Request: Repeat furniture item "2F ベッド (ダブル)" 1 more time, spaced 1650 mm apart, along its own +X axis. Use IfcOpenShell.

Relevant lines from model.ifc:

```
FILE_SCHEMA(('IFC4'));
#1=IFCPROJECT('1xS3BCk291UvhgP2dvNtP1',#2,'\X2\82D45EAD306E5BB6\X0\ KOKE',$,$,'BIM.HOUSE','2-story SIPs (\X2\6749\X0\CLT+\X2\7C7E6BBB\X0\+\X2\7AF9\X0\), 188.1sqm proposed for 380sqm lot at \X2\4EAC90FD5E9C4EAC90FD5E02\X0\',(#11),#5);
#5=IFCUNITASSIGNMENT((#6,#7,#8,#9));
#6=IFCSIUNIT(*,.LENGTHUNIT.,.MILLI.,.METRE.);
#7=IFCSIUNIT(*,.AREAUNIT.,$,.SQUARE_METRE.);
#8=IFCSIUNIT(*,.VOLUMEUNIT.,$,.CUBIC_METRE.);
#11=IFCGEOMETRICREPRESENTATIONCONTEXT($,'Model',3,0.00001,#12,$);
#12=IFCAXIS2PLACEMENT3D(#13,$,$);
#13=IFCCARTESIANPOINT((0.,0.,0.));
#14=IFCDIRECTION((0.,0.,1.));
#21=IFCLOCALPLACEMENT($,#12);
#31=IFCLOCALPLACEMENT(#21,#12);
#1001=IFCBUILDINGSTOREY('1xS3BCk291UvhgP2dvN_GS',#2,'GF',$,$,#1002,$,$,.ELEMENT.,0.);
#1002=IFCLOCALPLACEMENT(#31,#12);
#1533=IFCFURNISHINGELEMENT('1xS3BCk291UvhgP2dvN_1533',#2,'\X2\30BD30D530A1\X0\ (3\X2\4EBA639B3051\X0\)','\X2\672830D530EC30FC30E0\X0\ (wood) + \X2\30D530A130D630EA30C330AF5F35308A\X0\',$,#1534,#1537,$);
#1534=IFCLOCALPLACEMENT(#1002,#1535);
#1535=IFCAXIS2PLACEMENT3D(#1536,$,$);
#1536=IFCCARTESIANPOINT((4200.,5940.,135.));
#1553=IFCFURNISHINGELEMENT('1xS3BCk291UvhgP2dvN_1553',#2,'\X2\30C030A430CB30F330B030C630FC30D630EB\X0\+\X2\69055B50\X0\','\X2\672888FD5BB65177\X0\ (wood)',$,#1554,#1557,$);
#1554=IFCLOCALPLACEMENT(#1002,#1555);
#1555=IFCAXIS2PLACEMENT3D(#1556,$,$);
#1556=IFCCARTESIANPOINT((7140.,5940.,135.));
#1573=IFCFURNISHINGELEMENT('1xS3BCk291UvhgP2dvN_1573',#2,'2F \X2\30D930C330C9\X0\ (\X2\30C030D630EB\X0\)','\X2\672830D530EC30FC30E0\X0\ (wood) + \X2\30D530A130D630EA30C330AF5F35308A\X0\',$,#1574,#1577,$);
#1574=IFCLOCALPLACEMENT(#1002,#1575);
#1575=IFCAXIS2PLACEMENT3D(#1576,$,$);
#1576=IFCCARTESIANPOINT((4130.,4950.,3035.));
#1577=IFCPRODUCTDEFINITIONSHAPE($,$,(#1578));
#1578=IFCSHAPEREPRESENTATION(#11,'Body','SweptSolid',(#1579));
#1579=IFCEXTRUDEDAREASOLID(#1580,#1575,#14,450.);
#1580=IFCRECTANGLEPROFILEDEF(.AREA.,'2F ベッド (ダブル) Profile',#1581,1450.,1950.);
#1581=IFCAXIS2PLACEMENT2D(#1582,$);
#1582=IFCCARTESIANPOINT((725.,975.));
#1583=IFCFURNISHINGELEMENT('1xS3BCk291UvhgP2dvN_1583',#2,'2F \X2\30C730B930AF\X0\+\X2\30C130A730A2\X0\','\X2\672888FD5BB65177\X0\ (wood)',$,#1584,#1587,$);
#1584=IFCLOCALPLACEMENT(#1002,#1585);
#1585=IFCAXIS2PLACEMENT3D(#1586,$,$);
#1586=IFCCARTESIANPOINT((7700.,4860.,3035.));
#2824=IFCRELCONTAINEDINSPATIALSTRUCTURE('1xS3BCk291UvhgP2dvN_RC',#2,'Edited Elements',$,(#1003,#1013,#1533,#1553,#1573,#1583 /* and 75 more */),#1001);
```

```python
import ifcopenshell
import ifcopenshell.api.geometry
import ifcopenshell.api.root
import ifcopenshell.util.element
import ifcopenshell.util.placement

model = ifcopenshell.open("model.ifc")


def reuse_history(source, copy):
    """copy_class also copies each property set's owner history, people and application; keep the originals."""
    for rel in copy.IsDefinedBy:
        if rel.is_a("IfcRelDefinesByProperties") and (history := rel.RelatingPropertyDefinition.OwnerHistory):
            rel.RelatingPropertyDefinition.OwnerHistory = source.OwnerHistory
            ifcopenshell.util.element.remove_deep2(model, history)


source = model.by_guid("1xS3BCk291UvhgP2dvN_1573")
base = ifcopenshell.util.placement.get_local_placement(source.ObjectPlacement)
step = base[:3, 0] * 1650.0

for i in range(1, 2):
    copy = ifcopenshell.api.root.copy_class(model, product=source)
    copy.Representation = ifcopenshell.util.element.copy_deep(
        model, source.Representation, exclude=["IfcGeometricRepresentationContext", "IfcRepresentationMap"]
    )
    reuse_history(source, copy)
    matrix = base.copy()
    matrix[:3, 3] += i * step
    print("added at", matrix[:3, 3].round(3) + 0.0)
    ifcopenshell.api.geometry.edit_object_placement(model, product=copy, matrix=matrix, is_si=False)

model.write("model_updated.ifc")
```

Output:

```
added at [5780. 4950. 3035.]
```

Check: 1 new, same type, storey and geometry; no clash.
